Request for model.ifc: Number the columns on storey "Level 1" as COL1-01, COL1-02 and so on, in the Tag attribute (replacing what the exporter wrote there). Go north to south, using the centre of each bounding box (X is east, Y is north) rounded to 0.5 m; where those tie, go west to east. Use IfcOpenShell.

First a look at what the model holds.

```python
import ifcopenshell
import ifcopenshell.util.element
import ifcopenshell.util.placement

model = ifcopenshell.open("model.ifc")
print(model.schema)
storey = next(s for s in model.by_type("IfcBuildingStorey") if s.Name == "Level 1")
columns = [e for e in ifcopenshell.util.element.get_decomposition(storey) if e.is_a("IfcColumn")]
for e in sorted(columns, key=lambda e: e.id()):
    origin = ifcopenshell.util.placement.get_local_placement(e.ObjectPlacement)[:3, 3]
    print(e.id(), e.Tag, e.Name, origin.round(2) + 0.0, sep=" | ")
```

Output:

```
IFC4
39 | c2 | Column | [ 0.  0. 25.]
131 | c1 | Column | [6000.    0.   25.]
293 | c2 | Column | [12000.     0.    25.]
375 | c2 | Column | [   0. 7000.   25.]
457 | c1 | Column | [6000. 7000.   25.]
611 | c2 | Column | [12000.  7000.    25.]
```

```python
import ifcopenshell
import ifcopenshell.geom
import ifcopenshell.util.element
import ifcopenshell.util.shape

model = ifcopenshell.open("model.ifc")
settings = ifcopenshell.geom.settings()
settings.set("use-world-coords", True)


def centre(element):
    shape = ifcopenshell.geom.create_shape(settings, element)
    return ifcopenshell.util.shape.get_bbox_centroid(shape.geometry)


storey = next(s for s in model.by_type("IfcBuildingStorey") if s.Name == "Level 1")
columns = [e for e in ifcopenshell.util.element.get_decomposition(storey) if e.is_a("IfcColumn")]

# Insertion points can sit at a corner or the storey origin, so sort by the geometry (in metres).
centres = {e: centre(e) for e in columns}
columns.sort(key=lambda e: (-round(centres[e][1] / 0.5), centres[e][0]))

for i, e in enumerate(columns, start=1):
    number = f"COL1-{i:02d}"
    e.Tag = number
    print(e.id(), number)

model.write("model_v2.ifc")
```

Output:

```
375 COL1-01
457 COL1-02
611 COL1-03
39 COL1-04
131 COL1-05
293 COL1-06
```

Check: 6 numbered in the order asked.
